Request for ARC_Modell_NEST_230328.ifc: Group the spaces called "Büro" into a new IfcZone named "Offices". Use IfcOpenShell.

First a look at what the model holds.

```python
import ifcopenshell

model = ifcopenshell.open("ARC_Modell_NEST_230328.ifc")
print(model.schema)
seen = {}
for space in model.by_type("IfcSpace"):
    seen[space.LongName] = seen.get(space.LongName, 0) + 1
for name, count in sorted(seen.items(), key=str):
    print(count, "x", name)
print("zones:", [z.Name for z in model.by_type("IfcZone")][:20])
```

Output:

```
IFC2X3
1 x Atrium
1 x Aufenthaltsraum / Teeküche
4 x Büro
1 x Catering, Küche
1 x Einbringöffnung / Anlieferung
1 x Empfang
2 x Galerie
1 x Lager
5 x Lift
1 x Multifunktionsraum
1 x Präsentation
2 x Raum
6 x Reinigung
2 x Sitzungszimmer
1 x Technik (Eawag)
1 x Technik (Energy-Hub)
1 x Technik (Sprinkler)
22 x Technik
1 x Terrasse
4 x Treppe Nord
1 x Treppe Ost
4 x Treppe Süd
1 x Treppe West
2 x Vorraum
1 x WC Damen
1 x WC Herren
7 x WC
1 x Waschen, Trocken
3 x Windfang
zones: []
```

```python
import ifcopenshell
import ifcopenshell.api.group
import ifcopenshell.api.root

model = ifcopenshell.open("ARC_Modell_NEST_230328.ifc")

names = {"Büro"}
spaces = [s for s in model.by_type("IfcSpace") if s.LongName in names]

zone = ifcopenshell.api.root.create_entity(model, ifc_class="IfcZone", name="Offices")
ifcopenshell.api.group.assign_group(model, products=spaces, group=zone)
print(len(spaces), "spaces in", zone.Name)

model.write("ARC_Modell_NEST_230328-out.ifc")
```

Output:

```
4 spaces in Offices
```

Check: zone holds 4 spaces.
